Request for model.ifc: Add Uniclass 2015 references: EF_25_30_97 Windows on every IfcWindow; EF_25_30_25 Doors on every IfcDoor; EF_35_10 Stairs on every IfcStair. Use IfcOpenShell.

First a look at what the model holds.

```python
import ifcopenshell

model = ifcopenshell.open("model.ifc")
print(model.schema)
print("classifications:", [c.Name for c in model.by_type("IfcClassification")])
for ifc_class in ("IfcDoor", "IfcRoof", "IfcStair", "IfcWall", "IfcWindow"):
    print(ifc_class, len(model.by_type(ifc_class)))
```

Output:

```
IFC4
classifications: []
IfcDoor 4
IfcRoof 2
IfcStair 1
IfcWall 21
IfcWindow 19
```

```python
import ifcopenshell
import ifcopenshell.api.classification

model = ifcopenshell.open("model.ifc")

system = ifcopenshell.api.classification.add_classification(model, classification="Uniclass 2015")

codes = {
    "IfcWindow": ("EF_25_30_97", "Windows"),
    "IfcDoor": ("EF_25_30_25", "Doors"),
    "IfcStair": ("EF_35_10", "Stairs"),
}
for ifc_class, (code, name) in codes.items():
    products = model.by_type(ifc_class)
    ifcopenshell.api.classification.add_reference(
        model, products=products, classification=system, identification=code, name=name
    )
    print(code, len(products))

model.write("model_edited.ifc")
```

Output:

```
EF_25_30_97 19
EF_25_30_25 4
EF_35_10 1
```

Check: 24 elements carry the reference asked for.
